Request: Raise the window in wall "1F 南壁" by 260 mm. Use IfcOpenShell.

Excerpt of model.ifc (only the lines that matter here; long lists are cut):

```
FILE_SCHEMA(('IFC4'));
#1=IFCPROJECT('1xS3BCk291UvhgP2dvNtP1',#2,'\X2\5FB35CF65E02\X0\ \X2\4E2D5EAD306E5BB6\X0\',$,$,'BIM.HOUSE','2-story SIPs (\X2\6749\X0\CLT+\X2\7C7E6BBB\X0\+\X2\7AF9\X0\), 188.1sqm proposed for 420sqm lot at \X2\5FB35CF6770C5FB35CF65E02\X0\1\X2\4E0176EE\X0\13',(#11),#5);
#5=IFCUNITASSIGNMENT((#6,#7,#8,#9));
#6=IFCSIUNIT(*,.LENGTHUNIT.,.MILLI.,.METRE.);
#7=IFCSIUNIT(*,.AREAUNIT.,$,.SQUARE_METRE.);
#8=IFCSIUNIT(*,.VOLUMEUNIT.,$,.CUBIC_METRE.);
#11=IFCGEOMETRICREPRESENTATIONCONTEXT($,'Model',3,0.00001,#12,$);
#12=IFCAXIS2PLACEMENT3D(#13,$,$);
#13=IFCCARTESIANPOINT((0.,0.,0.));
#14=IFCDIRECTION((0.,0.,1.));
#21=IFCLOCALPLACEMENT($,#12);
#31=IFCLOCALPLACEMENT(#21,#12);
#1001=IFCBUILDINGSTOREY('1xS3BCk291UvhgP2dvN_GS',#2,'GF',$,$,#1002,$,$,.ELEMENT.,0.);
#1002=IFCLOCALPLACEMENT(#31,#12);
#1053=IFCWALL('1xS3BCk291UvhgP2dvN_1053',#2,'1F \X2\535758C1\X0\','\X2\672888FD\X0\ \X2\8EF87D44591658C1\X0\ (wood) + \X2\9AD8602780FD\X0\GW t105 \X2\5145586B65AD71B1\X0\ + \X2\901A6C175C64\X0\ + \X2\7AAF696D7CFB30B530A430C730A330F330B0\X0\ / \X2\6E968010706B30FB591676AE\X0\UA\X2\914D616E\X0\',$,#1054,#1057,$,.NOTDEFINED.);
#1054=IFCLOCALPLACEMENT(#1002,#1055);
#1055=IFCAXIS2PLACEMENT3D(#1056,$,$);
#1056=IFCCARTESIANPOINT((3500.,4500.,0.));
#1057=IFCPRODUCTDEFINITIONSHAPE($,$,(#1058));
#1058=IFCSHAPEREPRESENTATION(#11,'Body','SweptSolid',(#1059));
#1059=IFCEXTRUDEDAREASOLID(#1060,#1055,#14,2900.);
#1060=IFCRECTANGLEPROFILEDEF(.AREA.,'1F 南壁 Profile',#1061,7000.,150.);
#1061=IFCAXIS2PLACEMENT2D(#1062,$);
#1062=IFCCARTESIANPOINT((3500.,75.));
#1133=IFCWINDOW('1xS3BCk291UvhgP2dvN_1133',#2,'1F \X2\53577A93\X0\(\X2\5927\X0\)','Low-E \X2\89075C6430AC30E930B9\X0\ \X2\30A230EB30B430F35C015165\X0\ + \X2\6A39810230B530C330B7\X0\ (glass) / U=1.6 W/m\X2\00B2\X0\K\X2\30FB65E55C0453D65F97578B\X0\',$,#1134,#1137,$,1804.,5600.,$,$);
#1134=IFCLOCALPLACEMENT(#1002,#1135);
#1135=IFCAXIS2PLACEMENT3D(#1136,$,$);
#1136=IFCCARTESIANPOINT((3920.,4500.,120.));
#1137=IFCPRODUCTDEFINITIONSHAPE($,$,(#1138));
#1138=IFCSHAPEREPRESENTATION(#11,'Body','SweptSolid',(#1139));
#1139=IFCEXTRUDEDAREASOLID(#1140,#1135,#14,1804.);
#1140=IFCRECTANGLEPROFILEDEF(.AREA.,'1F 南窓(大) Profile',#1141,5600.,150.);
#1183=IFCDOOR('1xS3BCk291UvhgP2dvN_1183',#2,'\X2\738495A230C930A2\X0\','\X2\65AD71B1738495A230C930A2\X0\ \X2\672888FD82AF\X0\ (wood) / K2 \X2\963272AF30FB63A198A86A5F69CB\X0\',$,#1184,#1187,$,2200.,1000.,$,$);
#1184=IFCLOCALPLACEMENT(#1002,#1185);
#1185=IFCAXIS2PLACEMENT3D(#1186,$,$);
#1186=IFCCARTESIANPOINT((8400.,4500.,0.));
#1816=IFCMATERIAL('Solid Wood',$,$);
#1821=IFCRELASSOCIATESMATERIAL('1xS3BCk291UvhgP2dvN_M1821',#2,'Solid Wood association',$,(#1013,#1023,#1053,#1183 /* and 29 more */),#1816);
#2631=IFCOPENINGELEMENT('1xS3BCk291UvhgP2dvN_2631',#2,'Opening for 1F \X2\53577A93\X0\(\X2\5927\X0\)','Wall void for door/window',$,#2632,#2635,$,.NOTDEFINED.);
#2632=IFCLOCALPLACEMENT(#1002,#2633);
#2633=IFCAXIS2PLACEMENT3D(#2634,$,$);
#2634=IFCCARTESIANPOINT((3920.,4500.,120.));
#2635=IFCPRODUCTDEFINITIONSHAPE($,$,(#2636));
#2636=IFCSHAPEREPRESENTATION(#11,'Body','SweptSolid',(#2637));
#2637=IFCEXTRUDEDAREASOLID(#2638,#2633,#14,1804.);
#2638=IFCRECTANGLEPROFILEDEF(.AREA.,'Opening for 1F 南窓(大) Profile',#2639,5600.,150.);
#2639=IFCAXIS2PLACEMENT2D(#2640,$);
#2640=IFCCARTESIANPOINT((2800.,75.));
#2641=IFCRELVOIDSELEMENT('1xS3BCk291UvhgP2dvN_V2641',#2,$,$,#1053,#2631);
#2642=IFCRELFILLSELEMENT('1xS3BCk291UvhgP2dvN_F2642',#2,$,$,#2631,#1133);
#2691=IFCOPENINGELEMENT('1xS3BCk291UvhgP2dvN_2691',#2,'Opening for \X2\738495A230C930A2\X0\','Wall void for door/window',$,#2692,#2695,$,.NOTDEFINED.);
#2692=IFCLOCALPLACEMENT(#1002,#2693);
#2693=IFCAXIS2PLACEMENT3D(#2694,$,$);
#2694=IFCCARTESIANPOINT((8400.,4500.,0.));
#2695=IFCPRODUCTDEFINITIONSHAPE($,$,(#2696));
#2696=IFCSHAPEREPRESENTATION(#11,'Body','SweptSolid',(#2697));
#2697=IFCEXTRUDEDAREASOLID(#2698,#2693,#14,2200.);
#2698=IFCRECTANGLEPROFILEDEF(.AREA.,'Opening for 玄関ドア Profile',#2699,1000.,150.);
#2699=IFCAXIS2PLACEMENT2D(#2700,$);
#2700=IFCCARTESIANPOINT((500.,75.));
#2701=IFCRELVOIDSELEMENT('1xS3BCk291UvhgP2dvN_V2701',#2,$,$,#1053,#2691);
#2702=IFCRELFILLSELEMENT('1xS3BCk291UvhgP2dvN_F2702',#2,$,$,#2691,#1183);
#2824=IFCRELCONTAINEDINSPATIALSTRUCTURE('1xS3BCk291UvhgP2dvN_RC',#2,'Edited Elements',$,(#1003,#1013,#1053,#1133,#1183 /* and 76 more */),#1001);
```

```python
import numpy as np
import ifcopenshell
import ifcopenshell.api.geometry
import ifcopenshell.util.placement
import ifcopenshell.util.unit

model = ifcopenshell.open("model.ifc")
unit_scale = ifcopenshell.util.unit.calculate_unit_scale(model)

window = model.by_guid("1xS3BCk291UvhgP2dvN_1133")
opening = window.FillsVoids[0].RelatingOpeningElement
dz = 260.0

shift = np.array([0.0, 0.0, dz])
# The window is not placed relative to its opening, so move both.
for product in (opening, window):
    matrix = ifcopenshell.util.placement.get_local_placement(product.ObjectPlacement)
    matrix[:3, 3] += shift
    ifcopenshell.api.geometry.edit_object_placement(model, product=product, matrix=matrix, is_si=False)

print(f"moved by {dz * unit_scale:+.3f} m")

model.write("model-out.ifc")
```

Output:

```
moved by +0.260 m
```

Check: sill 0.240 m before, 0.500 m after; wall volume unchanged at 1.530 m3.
